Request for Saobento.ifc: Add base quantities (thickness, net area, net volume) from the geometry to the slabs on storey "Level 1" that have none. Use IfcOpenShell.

First a look at what the model holds.

```python
import ifcopenshell
import ifcopenshell.util.element
import ifcopenshell.util.unit

model = ifcopenshell.open("Saobento.ifc")
print(model.schema)
for unit_type in ("LENGTHUNIT", "AREAUNIT", "VOLUMEUNIT"):
    print(unit_type, ifcopenshell.util.unit.calculate_unit_scale(model, unit_type))
storey = next(s for s in model.by_type("IfcBuildingStorey") if s.Name == "Level 1")
slabs = [e for e in ifcopenshell.util.element.get_decomposition(storey) if e.is_a("IfcSlab")]
for e in sorted(slabs, key=lambda e: e.id()):
    print(e.id(), e.is_a(), e.Name, list(ifcopenshell.util.element.get_psets(e, qtos_only=True)), sep=" | ")
```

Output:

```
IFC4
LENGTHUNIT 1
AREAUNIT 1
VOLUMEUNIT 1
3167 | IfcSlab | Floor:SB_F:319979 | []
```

```python
import ifcopenshell
import ifcopenshell.api.pset
import ifcopenshell.geom
import ifcopenshell.util.element
import ifcopenshell.util.shape
import ifcopenshell.util.unit

model = ifcopenshell.open("Saobento.ifc")
unit_scale = ifcopenshell.util.unit.calculate_unit_scale(model)
area_scale = ifcopenshell.util.unit.calculate_unit_scale(model, "AREAUNIT")
volume_scale = ifcopenshell.util.unit.calculate_unit_scale(model, "VOLUMEUNIT")
settings = ifcopenshell.geom.settings()

storey = next(s for s in model.by_type("IfcBuildingStorey") if s.Name == "Level 1")
slabs = [e for e in ifcopenshell.util.element.get_decomposition(storey) if e.is_a("IfcSlab")]

for e in sorted(slabs, key=lambda e: e.id()):
    if ifcopenshell.util.element.get_psets(e, qtos_only=True, should_inherit=False):
        continue
    # Geometry comes back in metres, in the element's own axes.
    shape = ifcopenshell.geom.create_shape(settings, e)
    values = {
        "Width": ifcopenshell.util.shape.get_z(shape.geometry) / unit_scale,
        "NetArea": ifcopenshell.util.shape.get_footprint_area(shape.geometry) / area_scale,
        "NetVolume": ifcopenshell.util.shape.get_volume(shape.geometry) / volume_scale,
    }
    qto = ifcopenshell.api.pset.add_qto(model, product=e, name="Qto_SlabBaseQuantities")
    ifcopenshell.api.pset.edit_qto(model, qto=qto, properties=values)
    print(e.id(), {k: round(v, 3) for k, v in values.items()})

model.write("Saobento_v2.ifc")
```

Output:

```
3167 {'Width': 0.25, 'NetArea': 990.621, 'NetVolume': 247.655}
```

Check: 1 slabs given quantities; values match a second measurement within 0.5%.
